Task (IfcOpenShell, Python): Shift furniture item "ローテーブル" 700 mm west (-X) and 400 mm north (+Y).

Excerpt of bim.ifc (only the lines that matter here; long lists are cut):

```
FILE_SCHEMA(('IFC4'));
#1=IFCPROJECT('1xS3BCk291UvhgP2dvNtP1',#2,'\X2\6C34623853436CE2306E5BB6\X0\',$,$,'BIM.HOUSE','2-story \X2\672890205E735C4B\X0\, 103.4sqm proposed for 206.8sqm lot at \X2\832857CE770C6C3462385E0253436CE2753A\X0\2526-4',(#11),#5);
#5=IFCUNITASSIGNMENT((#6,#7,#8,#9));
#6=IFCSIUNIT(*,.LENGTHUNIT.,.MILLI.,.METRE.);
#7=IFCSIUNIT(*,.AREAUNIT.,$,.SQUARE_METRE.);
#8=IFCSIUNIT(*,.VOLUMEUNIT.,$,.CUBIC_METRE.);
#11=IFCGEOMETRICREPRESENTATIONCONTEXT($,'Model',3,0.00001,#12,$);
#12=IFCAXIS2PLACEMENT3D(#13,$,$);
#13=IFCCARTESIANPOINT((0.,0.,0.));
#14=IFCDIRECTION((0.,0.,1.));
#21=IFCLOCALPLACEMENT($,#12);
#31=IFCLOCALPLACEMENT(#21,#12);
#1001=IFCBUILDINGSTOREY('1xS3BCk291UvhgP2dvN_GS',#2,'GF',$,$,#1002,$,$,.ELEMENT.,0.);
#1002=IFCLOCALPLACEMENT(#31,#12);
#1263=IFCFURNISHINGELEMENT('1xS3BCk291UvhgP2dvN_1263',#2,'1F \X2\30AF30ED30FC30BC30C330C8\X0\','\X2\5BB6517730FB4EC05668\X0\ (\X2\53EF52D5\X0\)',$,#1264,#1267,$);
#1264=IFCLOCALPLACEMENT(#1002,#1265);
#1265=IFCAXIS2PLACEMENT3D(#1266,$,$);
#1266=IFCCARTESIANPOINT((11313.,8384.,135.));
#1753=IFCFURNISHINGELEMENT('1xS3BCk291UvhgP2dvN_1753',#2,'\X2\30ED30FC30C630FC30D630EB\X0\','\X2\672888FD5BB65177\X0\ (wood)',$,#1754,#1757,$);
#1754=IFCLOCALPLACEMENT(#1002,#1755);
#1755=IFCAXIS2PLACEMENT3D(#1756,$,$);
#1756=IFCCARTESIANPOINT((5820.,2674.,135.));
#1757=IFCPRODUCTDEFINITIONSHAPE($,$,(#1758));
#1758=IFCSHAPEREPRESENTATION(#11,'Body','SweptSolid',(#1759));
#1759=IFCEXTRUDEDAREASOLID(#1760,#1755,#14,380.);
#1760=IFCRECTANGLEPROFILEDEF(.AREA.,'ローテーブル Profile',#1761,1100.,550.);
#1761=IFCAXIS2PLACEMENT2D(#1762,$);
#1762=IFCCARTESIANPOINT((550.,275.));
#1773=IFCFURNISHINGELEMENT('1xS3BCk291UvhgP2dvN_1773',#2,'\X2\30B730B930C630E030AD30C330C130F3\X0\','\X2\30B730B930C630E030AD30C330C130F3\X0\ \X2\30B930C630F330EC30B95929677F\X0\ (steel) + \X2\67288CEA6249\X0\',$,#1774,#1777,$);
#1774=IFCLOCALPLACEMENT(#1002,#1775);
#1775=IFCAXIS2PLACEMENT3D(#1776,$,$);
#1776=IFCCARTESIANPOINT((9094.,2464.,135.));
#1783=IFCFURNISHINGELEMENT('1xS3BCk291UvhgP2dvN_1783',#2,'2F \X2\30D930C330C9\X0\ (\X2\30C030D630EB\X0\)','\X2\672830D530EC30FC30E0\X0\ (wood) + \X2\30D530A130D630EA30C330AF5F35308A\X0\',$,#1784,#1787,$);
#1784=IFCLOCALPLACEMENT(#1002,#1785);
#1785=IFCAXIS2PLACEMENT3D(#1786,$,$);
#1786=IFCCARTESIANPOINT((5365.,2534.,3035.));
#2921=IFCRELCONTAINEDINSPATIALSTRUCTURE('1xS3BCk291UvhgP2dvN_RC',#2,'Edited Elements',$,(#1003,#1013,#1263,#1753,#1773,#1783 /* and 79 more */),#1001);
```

```python
import ifcopenshell
import ifcopenshell.api.geometry
import ifcopenshell.util.placement
import ifcopenshell.util.unit

model = ifcopenshell.open("bim.ifc")
unit_scale = ifcopenshell.util.unit.calculate_unit_scale(model)

item = model.by_guid("1xS3BCk291UvhgP2dvN_1753")
matrix = ifcopenshell.util.placement.get_local_placement(item.ObjectPlacement)
matrix[0, 3] -= 0.7 / unit_scale
matrix[1, 3] += 0.4 / unit_scale
ifcopenshell.api.geometry.edit_object_placement(model, product=item, matrix=matrix, is_si=False)

print(ifcopenshell.util.placement.get_local_placement(item.ObjectPlacement).round(3) + 0.0)

model.write("bim_edited.ifc")
```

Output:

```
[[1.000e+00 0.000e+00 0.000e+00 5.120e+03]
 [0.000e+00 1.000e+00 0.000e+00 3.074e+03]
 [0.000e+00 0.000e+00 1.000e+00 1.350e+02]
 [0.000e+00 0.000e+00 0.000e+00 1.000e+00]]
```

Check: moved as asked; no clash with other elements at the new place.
